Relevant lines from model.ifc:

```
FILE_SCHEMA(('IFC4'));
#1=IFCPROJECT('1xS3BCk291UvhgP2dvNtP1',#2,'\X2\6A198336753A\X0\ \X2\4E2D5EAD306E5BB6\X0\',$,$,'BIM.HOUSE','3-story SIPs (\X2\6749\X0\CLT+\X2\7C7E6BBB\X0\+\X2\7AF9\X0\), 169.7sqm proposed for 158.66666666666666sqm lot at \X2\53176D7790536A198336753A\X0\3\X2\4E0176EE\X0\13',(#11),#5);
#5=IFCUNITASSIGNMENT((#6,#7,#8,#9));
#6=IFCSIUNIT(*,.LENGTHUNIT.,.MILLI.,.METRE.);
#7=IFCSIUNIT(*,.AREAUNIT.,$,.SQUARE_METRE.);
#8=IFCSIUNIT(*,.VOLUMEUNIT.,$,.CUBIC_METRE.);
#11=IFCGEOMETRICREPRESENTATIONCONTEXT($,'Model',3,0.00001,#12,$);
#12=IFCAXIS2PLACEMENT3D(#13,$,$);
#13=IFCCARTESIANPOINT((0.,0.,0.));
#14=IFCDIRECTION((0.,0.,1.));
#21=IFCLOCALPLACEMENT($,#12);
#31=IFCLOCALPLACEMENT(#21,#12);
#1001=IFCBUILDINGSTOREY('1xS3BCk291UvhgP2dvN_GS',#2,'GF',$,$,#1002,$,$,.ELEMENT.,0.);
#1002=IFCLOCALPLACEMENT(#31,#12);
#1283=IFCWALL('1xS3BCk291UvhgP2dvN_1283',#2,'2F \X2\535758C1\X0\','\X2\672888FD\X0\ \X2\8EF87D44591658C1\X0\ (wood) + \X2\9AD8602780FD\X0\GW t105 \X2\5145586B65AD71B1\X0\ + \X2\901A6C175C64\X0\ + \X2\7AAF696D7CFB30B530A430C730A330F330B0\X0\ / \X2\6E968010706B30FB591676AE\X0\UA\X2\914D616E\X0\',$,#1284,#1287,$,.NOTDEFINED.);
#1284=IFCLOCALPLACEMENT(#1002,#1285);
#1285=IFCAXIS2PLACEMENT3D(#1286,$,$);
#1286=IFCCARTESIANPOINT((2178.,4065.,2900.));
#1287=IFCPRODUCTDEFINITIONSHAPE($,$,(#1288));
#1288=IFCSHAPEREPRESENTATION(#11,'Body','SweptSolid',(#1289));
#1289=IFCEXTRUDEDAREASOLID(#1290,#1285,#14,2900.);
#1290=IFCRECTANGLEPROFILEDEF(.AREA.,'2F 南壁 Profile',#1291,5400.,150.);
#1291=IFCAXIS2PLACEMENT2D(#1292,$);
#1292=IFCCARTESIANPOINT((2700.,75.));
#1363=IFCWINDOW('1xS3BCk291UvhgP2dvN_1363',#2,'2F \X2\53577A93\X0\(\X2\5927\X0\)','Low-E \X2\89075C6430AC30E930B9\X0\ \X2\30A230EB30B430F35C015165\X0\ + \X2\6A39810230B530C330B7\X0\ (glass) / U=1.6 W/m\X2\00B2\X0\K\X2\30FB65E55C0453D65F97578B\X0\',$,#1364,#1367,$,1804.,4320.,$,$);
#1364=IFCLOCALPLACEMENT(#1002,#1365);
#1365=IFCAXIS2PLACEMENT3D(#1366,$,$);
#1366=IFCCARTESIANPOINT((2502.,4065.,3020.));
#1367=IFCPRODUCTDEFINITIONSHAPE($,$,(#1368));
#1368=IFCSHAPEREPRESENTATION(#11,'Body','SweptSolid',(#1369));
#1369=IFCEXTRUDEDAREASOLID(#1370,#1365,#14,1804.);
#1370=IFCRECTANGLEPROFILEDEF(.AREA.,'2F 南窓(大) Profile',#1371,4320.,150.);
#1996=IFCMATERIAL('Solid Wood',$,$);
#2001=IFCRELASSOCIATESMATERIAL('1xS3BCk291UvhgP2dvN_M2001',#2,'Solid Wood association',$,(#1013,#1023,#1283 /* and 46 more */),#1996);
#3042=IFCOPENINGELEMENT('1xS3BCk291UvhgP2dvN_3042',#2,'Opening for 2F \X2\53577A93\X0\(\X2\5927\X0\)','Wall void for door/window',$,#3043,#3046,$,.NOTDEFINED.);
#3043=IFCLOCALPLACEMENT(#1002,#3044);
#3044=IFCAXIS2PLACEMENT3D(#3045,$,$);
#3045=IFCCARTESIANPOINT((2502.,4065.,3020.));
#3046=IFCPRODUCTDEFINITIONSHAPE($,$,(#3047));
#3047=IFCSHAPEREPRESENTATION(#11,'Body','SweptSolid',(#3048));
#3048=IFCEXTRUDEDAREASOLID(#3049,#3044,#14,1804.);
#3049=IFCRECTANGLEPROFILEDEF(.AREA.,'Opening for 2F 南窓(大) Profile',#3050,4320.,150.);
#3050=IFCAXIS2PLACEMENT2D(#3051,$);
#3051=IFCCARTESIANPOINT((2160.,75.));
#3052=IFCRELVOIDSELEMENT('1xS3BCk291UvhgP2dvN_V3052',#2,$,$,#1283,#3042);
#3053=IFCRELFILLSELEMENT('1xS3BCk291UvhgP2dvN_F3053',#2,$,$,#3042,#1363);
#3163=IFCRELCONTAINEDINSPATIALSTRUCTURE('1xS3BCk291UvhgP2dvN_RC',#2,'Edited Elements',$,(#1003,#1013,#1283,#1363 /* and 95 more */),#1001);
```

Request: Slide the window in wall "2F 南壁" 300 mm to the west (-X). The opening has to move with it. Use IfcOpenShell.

```python
import ifcopenshell
import ifcopenshell.api.geometry
import ifcopenshell.util.placement
import ifcopenshell.util.unit

model = ifcopenshell.open("model.ifc")
unit_scale = ifcopenshell.util.unit.calculate_unit_scale(model)

window = model.by_id(1363)
opening = window.FillsVoids[0].RelatingOpeningElement
wall = opening.VoidsElements[0].RelatingBuildingElement

wall_matrix = ifcopenshell.util.placement.get_local_placement(wall.ObjectPlacement)
shift = wall_matrix[:3, 0] * -0.3 / unit_scale
before = ifcopenshell.util.placement.get_local_placement(window.ObjectPlacement)[:3, 3].copy()

# The window is not placed relative to its opening, so move both.
for product in (opening, window):
    matrix = ifcopenshell.util.placement.get_local_placement(product.ObjectPlacement)
    matrix[:3, 3] += shift
    ifcopenshell.api.geometry.edit_object_placement(model, product=product, matrix=matrix, is_si=False)

after = ifcopenshell.util.placement.get_local_placement(window.ObjectPlacement)[:3, 3]
print("window moved by", (after - before).round(3) + 0.0)

model.write("model_edited.ifc")
```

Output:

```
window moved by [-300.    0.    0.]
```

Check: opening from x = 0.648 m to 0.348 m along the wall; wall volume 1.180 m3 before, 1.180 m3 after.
